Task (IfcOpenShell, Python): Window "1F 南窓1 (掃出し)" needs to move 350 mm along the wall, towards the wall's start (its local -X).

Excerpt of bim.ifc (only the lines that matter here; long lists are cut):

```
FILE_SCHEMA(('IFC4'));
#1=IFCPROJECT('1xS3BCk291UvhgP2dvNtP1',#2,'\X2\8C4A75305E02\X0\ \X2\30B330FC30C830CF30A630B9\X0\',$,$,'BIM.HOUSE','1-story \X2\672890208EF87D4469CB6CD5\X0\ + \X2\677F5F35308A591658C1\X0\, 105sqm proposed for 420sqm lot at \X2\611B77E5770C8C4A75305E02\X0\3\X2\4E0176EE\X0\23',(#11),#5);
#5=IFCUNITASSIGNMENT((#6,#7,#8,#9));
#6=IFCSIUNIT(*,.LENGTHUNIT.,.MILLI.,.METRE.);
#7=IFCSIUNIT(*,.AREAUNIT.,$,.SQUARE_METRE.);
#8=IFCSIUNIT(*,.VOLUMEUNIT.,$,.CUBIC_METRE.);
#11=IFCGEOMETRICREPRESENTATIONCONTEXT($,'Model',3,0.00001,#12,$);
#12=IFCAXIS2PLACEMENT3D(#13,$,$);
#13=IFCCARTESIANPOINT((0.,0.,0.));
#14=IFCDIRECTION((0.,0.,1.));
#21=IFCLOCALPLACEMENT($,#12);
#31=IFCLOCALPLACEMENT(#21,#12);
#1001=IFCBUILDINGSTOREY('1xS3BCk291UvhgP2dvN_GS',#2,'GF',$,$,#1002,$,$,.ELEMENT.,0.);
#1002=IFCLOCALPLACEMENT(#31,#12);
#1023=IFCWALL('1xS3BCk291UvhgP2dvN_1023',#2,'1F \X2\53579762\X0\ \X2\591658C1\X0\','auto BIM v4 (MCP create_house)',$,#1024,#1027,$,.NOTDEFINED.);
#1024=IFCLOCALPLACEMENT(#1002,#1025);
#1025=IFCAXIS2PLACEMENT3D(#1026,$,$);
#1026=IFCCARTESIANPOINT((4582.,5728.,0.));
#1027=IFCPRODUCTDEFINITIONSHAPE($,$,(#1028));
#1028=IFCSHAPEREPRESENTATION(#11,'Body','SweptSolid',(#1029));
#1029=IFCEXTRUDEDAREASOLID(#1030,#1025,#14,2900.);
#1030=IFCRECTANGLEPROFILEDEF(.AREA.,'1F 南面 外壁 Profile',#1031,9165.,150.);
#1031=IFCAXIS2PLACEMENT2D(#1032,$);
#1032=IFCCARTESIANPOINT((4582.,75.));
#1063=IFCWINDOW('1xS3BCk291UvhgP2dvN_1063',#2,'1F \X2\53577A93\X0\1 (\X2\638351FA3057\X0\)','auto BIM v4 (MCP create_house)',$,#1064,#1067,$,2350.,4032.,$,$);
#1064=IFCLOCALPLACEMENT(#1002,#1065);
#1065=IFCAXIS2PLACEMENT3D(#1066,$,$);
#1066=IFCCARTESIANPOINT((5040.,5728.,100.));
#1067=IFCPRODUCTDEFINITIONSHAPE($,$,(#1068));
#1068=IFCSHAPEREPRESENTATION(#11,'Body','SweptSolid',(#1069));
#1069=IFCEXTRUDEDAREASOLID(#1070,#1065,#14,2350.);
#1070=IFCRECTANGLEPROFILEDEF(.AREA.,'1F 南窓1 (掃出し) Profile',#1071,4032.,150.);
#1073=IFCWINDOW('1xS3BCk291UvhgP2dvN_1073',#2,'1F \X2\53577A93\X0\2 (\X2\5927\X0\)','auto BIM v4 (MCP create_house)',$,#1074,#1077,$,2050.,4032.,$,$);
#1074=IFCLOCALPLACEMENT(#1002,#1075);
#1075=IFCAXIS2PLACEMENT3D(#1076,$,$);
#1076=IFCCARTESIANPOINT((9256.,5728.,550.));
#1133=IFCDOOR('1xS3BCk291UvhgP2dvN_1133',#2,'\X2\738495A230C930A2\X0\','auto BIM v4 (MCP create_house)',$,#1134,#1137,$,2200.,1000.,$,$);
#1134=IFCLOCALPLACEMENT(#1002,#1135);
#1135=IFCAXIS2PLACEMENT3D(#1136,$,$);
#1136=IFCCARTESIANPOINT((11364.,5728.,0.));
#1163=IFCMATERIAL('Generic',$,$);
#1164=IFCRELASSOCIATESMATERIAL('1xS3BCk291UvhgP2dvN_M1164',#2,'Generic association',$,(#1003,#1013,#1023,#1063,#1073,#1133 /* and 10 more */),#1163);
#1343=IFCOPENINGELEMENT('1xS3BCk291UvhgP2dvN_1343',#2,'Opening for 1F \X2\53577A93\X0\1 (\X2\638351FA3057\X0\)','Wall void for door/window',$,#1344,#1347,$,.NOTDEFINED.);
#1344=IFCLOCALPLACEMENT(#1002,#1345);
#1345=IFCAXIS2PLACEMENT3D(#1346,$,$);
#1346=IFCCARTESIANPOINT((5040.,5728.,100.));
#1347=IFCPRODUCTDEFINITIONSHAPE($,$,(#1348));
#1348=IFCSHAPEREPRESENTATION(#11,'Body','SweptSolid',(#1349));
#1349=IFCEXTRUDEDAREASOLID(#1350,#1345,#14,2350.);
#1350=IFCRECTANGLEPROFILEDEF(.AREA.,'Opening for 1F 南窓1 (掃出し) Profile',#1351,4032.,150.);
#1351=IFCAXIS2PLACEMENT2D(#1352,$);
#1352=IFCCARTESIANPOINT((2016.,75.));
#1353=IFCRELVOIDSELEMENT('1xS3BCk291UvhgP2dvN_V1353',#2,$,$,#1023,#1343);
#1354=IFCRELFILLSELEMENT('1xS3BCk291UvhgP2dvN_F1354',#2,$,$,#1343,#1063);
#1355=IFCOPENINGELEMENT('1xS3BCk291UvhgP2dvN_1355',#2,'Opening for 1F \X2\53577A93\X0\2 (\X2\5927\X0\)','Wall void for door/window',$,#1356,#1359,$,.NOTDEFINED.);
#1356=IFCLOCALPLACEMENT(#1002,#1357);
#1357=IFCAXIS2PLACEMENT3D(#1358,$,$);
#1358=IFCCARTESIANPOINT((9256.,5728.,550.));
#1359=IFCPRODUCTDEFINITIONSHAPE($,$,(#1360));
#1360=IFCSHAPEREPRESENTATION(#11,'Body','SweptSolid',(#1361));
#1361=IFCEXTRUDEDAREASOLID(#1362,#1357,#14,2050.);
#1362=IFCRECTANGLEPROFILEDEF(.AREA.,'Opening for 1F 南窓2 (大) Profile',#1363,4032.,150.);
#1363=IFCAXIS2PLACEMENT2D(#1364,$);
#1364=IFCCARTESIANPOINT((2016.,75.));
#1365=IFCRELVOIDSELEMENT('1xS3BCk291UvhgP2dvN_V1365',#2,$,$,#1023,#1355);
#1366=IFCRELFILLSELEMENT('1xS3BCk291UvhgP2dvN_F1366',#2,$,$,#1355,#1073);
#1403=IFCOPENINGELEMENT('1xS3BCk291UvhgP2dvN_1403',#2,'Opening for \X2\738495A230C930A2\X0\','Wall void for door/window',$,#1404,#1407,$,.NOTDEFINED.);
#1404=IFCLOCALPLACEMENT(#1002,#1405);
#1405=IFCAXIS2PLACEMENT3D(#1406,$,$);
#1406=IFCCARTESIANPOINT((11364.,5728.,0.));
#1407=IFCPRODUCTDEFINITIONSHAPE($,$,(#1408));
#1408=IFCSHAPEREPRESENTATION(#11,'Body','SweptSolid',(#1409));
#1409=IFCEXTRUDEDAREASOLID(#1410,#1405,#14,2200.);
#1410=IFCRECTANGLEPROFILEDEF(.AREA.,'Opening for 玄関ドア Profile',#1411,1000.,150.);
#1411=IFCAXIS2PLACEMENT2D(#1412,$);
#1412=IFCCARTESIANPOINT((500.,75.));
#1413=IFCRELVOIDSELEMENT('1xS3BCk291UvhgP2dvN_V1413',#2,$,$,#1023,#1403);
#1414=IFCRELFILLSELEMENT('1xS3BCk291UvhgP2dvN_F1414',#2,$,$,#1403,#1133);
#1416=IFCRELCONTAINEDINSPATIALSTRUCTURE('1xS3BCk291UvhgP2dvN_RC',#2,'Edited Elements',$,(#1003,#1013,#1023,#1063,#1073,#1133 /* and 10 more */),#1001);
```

```python
import ifcopenshell
import ifcopenshell.api.geometry
import ifcopenshell.util.placement

model = ifcopenshell.open("bim.ifc")

window = model.by_guid("1xS3BCk291UvhgP2dvN_1063")
opening = window.FillsVoids[0].RelatingOpeningElement
wall = opening.VoidsElements[0].RelatingBuildingElement

wall_matrix = ifcopenshell.util.placement.get_local_placement(wall.ObjectPlacement)
shift = wall_matrix[:3, 0] * -350.0
before = ifcopenshell.util.placement.get_local_placement(window.ObjectPlacement)[:3, 3].copy()

# The window is not placed relative to its opening, so move both.
for product in (opening, window):
    matrix = ifcopenshell.util.placement.get_local_placement(product.ObjectPlacement)
    matrix[:3, 3] += shift
    ifcopenshell.api.geometry.edit_object_placement(model, product=product, matrix=matrix, is_si=False)

after = ifcopenshell.util.placement.get_local_placement(window.ObjectPlacement)[:3, 3]
print("window moved by", (after - before).round(3) + 0.0)

model.write("bim_v2.ifc")
```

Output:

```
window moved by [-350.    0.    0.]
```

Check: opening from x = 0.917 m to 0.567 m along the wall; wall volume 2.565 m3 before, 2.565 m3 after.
